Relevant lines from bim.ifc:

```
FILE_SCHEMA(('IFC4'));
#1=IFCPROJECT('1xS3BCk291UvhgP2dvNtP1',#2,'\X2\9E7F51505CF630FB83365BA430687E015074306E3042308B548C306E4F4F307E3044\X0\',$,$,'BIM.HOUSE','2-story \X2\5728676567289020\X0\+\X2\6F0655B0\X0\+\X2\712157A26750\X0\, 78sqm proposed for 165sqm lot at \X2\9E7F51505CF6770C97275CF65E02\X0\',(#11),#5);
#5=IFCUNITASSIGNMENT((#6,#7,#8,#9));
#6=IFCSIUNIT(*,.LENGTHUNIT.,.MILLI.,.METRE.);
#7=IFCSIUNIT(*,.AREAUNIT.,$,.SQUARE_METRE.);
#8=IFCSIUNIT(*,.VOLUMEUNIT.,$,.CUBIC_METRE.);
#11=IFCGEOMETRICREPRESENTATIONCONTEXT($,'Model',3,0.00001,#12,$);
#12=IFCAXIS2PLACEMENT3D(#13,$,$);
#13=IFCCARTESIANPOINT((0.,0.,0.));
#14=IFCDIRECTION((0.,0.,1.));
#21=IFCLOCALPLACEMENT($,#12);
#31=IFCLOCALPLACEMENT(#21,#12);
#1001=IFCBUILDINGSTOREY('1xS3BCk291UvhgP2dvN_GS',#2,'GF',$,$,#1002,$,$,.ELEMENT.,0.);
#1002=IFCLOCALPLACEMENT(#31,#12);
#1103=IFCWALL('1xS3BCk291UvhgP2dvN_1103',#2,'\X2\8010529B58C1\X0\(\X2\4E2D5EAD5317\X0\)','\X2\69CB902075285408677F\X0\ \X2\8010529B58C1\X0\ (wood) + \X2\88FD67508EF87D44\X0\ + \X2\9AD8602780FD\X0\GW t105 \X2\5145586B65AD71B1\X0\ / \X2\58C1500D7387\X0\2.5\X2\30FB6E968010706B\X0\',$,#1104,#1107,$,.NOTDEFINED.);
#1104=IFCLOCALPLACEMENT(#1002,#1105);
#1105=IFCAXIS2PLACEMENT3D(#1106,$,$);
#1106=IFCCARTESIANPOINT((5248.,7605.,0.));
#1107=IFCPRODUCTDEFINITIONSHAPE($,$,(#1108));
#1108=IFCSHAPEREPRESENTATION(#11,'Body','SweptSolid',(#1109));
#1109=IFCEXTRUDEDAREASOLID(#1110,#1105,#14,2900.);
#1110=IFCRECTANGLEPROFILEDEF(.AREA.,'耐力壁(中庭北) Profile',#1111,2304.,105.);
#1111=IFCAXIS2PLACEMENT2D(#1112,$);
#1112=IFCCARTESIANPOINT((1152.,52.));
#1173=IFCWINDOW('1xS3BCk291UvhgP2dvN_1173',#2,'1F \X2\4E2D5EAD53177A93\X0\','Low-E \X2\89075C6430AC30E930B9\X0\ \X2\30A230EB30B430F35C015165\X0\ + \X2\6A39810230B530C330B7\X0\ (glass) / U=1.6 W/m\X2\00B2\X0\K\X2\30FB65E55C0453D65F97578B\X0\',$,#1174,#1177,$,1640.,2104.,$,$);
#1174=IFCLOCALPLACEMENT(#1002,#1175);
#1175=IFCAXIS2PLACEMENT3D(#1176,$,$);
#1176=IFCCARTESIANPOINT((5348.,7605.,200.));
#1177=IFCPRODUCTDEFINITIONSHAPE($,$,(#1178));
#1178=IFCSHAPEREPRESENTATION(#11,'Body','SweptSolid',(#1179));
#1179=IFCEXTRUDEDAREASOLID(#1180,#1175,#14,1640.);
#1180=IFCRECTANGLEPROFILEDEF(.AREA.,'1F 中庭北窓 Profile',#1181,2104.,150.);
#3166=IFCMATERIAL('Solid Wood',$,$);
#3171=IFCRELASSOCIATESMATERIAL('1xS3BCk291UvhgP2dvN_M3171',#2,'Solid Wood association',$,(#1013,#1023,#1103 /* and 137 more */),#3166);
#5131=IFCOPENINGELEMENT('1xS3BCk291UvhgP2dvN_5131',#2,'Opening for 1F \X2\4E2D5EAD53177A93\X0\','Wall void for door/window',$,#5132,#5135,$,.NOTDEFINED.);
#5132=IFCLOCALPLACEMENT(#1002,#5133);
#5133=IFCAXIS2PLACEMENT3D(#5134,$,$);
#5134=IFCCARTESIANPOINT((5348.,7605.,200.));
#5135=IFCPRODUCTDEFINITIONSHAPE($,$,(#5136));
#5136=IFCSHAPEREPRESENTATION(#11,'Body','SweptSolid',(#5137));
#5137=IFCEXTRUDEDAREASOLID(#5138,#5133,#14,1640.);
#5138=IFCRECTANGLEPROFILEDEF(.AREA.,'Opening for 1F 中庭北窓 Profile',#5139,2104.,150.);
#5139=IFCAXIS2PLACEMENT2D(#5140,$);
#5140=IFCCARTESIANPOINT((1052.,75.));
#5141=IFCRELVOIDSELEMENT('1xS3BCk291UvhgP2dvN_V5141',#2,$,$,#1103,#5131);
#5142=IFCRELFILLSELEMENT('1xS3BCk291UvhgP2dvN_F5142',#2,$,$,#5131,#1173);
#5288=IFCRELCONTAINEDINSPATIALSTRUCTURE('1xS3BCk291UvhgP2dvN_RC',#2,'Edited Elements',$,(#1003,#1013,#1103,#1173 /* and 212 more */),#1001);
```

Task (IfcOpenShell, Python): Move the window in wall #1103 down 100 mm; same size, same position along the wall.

```python
import numpy as np
import ifcopenshell
import ifcopenshell.api.geometry
import ifcopenshell.util.placement
import ifcopenshell.util.unit

model = ifcopenshell.open("bim.ifc")
unit_scale = ifcopenshell.util.unit.calculate_unit_scale(model)

window = model.by_guid("1xS3BCk291UvhgP2dvN_1173")
opening = window.FillsVoids[0].RelatingOpeningElement
dz = -100.0

shift = np.array([0.0, 0.0, dz])
# The window is not placed relative to its opening, so move both.
for product in (opening, window):
    matrix = ifcopenshell.util.placement.get_local_placement(product.ObjectPlacement)
    matrix[:3, 3] += shift
    ifcopenshell.api.geometry.edit_object_placement(model, product=product, matrix=matrix, is_si=False)

print(f"moved by {dz * unit_scale:+.3f} m")

model.write("bim_v2.ifc")
```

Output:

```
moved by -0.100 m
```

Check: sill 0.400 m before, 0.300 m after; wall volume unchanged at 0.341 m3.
